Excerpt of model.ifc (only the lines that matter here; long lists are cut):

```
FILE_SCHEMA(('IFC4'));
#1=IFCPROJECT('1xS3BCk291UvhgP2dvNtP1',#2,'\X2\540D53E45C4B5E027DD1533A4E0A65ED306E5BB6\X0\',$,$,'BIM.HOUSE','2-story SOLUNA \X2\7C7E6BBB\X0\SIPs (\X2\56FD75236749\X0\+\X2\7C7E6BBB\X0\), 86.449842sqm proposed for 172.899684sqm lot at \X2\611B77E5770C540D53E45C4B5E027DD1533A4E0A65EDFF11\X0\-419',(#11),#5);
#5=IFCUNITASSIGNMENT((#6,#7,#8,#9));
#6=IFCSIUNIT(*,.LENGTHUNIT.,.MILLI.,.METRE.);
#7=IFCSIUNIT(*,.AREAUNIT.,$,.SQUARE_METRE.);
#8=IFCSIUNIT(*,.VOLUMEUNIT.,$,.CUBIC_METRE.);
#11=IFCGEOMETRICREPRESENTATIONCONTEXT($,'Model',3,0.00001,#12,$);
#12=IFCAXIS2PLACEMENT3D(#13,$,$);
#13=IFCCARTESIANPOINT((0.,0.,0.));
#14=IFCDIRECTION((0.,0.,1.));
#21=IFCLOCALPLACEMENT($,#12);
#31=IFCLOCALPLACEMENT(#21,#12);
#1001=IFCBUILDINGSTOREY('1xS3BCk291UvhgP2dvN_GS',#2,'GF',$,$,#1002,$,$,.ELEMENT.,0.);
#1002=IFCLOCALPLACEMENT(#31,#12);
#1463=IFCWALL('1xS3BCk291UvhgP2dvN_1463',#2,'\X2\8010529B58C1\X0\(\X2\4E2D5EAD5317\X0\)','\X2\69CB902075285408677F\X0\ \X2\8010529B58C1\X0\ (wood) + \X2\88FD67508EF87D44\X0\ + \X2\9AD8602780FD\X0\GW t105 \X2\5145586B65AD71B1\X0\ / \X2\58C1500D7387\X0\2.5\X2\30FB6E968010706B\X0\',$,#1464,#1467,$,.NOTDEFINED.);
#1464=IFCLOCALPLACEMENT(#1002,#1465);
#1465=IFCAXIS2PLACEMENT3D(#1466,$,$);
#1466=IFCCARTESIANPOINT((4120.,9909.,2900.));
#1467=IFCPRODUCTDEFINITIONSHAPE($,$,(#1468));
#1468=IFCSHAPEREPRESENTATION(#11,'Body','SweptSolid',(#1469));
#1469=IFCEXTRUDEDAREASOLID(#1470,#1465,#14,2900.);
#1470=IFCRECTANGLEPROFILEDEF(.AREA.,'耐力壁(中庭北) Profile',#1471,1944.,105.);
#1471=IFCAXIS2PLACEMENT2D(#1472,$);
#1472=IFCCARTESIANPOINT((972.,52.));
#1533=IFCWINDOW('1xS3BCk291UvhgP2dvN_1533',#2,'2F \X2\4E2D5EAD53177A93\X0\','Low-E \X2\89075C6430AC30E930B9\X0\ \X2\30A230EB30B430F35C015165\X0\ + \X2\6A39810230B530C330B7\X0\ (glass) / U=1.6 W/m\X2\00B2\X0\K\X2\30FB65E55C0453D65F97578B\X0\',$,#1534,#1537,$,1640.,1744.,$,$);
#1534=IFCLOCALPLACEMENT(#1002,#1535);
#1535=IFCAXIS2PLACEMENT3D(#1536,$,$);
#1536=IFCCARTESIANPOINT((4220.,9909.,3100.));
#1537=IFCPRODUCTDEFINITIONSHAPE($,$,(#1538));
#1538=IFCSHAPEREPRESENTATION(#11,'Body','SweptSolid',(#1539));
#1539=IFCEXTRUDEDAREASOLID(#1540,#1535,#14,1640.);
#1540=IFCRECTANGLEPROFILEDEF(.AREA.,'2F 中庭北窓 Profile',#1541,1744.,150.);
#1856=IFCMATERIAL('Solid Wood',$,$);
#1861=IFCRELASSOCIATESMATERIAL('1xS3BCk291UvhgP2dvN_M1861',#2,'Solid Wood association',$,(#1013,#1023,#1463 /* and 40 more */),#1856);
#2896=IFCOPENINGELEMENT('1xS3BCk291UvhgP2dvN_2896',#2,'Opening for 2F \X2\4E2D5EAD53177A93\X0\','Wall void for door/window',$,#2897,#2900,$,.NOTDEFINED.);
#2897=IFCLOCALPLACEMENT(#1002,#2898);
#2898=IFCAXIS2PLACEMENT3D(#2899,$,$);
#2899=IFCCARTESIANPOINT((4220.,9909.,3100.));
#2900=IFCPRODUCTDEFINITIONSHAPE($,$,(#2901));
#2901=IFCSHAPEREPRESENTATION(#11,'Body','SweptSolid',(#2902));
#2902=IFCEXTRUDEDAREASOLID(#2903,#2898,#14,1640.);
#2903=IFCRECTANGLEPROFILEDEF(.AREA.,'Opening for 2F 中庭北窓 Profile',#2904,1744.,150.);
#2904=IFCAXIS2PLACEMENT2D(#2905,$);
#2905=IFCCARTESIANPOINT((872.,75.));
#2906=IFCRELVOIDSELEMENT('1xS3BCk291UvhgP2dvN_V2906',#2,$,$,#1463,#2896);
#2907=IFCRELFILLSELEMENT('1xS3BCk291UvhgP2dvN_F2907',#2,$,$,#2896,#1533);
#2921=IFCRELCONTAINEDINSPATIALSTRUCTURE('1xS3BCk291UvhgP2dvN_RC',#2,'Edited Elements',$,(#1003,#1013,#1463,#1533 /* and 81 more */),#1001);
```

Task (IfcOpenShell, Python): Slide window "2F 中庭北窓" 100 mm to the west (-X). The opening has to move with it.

```python
import ifcopenshell
import ifcopenshell.api.geometry
import ifcopenshell.util.placement
import ifcopenshell.util.unit

model = ifcopenshell.open("model.ifc")
unit_scale = ifcopenshell.util.unit.calculate_unit_scale(model)

window = model.by_guid("1xS3BCk291UvhgP2dvN_1533")
opening = window.FillsVoids[0].RelatingOpeningElement
wall = opening.VoidsElements[0].RelatingBuildingElement

wall_matrix = ifcopenshell.util.placement.get_local_placement(wall.ObjectPlacement)
shift = wall_matrix[:3, 0] * -0.1 / unit_scale
before = ifcopenshell.util.placement.get_local_placement(window.ObjectPlacement)[:3, 3].copy()

# The window is not placed relative to its opening, so move both.
for product in (opening, window):
    matrix = ifcopenshell.util.placement.get_local_placement(product.ObjectPlacement)
    matrix[:3, 3] += shift
    ifcopenshell.api.geometry.edit_object_placement(model, product=product, matrix=matrix, is_si=False)

after = ifcopenshell.util.placement.get_local_placement(window.ObjectPlacement)[:3, 3]
print("window moved by", (after - before).round(3) + 0.0)

model.write("model_v2.ifc")
```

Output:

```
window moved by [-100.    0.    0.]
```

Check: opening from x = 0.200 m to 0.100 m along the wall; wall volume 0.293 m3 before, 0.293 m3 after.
